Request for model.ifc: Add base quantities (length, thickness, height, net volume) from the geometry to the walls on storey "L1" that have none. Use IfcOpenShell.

First a look at what the model holds.

```python
import ifcopenshell
import ifcopenshell.util.element
import ifcopenshell.util.unit

model = ifcopenshell.open("model.ifc")
print(model.schema)
for unit_type in ("LENGTHUNIT", "AREAUNIT", "VOLUMEUNIT"):
    print(unit_type, ifcopenshell.util.unit.calculate_unit_scale(model, unit_type))
storey = next(s for s in model.by_type("IfcBuildingStorey") if s.Name == "L1")
walls = [e for e in ifcopenshell.util.element.get_decomposition(storey) if e.is_a("IfcWall")]
for e in sorted(walls, key=lambda e: e.id()):
    print(e.id(), e.is_a(), e.Name, list(ifcopenshell.util.element.get_psets(e, qtos_only=True)), sep=" | ")
```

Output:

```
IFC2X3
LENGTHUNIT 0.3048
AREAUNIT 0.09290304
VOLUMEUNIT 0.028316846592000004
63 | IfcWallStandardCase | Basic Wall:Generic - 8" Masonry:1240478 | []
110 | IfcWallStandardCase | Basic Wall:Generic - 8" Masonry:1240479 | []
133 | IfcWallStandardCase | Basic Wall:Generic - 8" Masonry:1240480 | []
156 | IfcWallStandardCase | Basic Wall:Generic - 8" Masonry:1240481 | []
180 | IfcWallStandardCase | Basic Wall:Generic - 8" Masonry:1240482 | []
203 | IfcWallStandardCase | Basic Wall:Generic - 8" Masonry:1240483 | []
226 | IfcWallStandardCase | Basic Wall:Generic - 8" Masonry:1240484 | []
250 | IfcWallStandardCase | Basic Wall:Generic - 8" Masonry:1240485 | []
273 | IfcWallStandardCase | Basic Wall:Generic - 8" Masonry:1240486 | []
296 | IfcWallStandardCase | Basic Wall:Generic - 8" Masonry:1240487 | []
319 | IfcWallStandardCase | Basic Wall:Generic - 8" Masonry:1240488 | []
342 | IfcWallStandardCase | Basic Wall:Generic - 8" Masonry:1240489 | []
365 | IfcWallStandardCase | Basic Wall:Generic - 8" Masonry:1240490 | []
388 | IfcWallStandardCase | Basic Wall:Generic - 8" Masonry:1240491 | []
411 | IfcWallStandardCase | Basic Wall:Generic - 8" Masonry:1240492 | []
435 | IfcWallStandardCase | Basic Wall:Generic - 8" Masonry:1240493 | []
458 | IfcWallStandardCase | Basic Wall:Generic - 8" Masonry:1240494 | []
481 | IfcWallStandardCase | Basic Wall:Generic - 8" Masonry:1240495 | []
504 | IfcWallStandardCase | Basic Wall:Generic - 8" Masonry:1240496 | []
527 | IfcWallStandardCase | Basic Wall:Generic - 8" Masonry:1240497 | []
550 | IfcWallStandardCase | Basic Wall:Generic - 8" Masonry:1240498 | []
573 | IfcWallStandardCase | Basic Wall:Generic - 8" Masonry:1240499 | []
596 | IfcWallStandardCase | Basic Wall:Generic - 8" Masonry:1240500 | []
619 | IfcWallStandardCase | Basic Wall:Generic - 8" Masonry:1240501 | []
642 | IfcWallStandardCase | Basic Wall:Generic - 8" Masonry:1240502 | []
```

```python
import ifcopenshell
import ifcopenshell.api.pset
import ifcopenshell.geom
import ifcopenshell.util.element
import ifcopenshell.util.shape
import ifcopenshell.util.unit

model = ifcopenshell.open("model.ifc")
unit_scale = ifcopenshell.util.unit.calculate_unit_scale(model)
volume_scale = ifcopenshell.util.unit.calculate_unit_scale(model, "VOLUMEUNIT")
settings = ifcopenshell.geom.settings()

storey = next(s for s in model.by_type("IfcBuildingStorey") if s.Name == "L1")
walls = [e for e in ifcopenshell.util.element.get_decomposition(storey) if e.is_a("IfcWall")]

for e in sorted(walls, key=lambda e: e.id()):
    if ifcopenshell.util.element.get_psets(e, qtos_only=True, should_inherit=False):
        continue
    # Geometry comes back in metres, in the element's own axes.
    shape = ifcopenshell.geom.create_shape(settings, e)
    values = {
        "Length": ifcopenshell.util.shape.get_x(shape.geometry) / unit_scale,
        "Width": ifcopenshell.util.shape.get_y(shape.geometry) / unit_scale,
        "Height": ifcopenshell.util.shape.get_z(shape.geometry) / unit_scale,
        "NetVolume": ifcopenshell.util.shape.get_volume(shape.geometry) / volume_scale,
    }
    qto = ifcopenshell.api.pset.add_qto(model, product=e, name="BaseQuantities")
    ifcopenshell.api.pset.edit_qto(model, qto=qto, properties=values)
    print(e.id(), {k: round(v, 3) for k, v in values.items()})

model.write("model_v2.ifc")
```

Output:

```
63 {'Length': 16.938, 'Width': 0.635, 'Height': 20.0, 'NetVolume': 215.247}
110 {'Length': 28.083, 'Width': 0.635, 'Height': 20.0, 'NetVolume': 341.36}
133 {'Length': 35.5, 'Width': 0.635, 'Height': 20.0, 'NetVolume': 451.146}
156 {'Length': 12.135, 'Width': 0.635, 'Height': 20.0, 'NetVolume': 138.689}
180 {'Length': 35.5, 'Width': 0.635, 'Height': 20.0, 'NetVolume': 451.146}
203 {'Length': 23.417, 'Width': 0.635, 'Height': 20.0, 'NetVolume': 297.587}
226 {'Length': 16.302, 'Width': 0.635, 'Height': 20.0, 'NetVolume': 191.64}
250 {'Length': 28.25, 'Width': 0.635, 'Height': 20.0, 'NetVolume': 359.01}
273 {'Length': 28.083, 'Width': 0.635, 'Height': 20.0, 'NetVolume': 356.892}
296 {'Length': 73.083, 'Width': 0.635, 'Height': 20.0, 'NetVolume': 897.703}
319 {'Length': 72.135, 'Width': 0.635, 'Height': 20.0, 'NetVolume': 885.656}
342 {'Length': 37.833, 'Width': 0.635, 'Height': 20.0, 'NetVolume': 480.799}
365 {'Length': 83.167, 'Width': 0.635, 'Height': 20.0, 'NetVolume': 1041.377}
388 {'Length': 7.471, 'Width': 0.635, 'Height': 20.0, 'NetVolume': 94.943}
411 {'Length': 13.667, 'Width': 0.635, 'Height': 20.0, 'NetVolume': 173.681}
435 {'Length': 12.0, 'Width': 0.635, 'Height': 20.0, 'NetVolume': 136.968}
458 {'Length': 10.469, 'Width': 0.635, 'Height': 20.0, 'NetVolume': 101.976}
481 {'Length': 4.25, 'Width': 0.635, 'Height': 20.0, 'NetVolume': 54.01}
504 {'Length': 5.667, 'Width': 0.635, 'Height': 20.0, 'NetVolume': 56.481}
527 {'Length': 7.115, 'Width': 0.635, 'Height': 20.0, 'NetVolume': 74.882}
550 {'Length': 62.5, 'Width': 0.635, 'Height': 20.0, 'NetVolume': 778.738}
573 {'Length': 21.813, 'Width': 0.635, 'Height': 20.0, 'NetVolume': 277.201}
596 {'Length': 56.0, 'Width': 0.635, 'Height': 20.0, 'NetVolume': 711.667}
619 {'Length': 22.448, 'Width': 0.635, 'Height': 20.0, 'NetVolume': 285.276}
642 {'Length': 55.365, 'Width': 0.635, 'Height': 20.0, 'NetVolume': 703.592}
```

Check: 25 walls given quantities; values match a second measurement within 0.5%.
